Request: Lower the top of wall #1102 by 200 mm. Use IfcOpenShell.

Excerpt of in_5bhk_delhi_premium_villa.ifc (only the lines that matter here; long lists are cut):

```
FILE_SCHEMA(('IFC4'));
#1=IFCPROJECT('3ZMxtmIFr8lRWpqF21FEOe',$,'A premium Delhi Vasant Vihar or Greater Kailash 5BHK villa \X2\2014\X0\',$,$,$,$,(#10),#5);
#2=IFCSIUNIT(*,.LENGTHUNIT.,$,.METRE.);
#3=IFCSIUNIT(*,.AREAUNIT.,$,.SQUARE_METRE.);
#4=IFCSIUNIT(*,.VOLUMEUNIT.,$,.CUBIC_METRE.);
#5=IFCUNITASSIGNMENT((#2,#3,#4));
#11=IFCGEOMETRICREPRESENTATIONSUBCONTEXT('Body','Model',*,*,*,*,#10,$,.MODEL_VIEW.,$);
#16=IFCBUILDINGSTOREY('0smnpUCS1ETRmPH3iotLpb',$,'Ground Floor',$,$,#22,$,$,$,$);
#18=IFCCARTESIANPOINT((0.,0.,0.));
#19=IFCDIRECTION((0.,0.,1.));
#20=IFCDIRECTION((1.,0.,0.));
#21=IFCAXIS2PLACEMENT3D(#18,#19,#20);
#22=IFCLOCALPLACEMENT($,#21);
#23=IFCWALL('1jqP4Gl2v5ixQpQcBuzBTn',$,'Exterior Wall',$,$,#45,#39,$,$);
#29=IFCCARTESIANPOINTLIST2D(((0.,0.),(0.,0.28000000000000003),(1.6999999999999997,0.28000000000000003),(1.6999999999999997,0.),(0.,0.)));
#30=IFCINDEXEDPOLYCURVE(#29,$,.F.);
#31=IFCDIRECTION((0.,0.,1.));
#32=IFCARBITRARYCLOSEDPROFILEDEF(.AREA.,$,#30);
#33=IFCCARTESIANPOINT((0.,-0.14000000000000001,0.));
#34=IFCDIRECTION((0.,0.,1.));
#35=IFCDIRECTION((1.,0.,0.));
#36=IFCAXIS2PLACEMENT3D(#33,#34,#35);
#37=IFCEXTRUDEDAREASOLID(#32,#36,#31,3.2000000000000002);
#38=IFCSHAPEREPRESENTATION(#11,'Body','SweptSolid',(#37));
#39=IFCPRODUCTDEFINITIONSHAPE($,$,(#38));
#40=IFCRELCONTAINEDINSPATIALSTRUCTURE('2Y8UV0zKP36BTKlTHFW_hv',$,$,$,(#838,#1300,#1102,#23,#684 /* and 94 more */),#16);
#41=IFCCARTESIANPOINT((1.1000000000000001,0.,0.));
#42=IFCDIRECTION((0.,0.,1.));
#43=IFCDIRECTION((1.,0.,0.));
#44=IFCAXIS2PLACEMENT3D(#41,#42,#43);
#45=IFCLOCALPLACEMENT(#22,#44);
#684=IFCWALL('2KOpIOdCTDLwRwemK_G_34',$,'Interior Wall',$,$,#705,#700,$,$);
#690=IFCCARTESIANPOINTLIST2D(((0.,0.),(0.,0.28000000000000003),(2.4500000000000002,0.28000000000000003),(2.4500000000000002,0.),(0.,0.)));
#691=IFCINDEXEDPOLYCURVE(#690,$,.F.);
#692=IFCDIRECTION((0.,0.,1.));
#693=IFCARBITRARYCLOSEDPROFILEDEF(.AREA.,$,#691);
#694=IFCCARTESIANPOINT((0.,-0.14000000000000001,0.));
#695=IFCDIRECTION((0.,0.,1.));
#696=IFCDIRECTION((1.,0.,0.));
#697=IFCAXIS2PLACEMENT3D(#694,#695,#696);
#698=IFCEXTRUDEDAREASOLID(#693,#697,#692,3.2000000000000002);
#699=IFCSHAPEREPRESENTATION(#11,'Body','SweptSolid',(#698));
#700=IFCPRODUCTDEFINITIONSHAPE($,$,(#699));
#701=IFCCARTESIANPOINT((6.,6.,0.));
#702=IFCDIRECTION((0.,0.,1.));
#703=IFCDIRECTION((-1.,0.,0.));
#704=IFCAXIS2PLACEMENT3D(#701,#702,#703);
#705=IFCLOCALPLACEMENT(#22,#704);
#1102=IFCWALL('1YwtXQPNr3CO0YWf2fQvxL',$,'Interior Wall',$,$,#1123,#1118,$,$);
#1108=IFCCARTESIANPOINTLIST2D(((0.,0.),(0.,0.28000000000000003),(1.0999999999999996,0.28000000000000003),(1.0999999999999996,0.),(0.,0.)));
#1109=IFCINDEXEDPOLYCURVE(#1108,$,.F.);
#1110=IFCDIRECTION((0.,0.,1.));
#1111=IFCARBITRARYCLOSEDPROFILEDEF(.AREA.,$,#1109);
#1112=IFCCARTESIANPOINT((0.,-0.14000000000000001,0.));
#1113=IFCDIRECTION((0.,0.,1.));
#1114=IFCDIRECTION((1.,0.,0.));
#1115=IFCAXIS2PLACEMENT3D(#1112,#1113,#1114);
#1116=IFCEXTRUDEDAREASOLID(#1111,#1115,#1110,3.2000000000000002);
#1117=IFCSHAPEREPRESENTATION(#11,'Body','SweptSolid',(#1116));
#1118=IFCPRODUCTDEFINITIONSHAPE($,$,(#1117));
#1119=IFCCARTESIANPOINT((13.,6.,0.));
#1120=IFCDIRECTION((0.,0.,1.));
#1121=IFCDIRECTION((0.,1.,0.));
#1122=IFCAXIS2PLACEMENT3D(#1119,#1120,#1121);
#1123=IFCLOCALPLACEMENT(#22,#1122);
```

```python
import ifcopenshell
import ifcopenshell.geom
import ifcopenshell.util.representation
import ifcopenshell.util.shape
import ifcopenshell.util.unit

model = ifcopenshell.open("in_5bhk_delhi_premium_villa.ifc")
unit_scale = ifcopenshell.util.unit.calculate_unit_scale(model)
settings = ifcopenshell.geom.settings()


def volume(element):
    """Net volume in cubic metres, openings subtracted."""
    shape = ifcopenshell.geom.create_shape(settings, element)
    return ifcopenshell.util.shape.get_volume(shape.geometry)


wall = model.by_id(1102)
before = volume(wall)

body = ifcopenshell.util.representation.get_representation(wall, "Model", "Body")
solid = body.Items[0]
old_height = solid.Depth
solid.Depth -= 0.2 / unit_scale
after = volume(wall)

print(f"height {old_height:g} -> {solid.Depth:g}, volume {before:.3f} -> {after:.3f} m3")

model.write("in_5bhk_delhi_premium_villa-out.ifc")
```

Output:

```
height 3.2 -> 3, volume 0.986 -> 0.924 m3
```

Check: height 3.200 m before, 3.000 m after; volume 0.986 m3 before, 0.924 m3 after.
